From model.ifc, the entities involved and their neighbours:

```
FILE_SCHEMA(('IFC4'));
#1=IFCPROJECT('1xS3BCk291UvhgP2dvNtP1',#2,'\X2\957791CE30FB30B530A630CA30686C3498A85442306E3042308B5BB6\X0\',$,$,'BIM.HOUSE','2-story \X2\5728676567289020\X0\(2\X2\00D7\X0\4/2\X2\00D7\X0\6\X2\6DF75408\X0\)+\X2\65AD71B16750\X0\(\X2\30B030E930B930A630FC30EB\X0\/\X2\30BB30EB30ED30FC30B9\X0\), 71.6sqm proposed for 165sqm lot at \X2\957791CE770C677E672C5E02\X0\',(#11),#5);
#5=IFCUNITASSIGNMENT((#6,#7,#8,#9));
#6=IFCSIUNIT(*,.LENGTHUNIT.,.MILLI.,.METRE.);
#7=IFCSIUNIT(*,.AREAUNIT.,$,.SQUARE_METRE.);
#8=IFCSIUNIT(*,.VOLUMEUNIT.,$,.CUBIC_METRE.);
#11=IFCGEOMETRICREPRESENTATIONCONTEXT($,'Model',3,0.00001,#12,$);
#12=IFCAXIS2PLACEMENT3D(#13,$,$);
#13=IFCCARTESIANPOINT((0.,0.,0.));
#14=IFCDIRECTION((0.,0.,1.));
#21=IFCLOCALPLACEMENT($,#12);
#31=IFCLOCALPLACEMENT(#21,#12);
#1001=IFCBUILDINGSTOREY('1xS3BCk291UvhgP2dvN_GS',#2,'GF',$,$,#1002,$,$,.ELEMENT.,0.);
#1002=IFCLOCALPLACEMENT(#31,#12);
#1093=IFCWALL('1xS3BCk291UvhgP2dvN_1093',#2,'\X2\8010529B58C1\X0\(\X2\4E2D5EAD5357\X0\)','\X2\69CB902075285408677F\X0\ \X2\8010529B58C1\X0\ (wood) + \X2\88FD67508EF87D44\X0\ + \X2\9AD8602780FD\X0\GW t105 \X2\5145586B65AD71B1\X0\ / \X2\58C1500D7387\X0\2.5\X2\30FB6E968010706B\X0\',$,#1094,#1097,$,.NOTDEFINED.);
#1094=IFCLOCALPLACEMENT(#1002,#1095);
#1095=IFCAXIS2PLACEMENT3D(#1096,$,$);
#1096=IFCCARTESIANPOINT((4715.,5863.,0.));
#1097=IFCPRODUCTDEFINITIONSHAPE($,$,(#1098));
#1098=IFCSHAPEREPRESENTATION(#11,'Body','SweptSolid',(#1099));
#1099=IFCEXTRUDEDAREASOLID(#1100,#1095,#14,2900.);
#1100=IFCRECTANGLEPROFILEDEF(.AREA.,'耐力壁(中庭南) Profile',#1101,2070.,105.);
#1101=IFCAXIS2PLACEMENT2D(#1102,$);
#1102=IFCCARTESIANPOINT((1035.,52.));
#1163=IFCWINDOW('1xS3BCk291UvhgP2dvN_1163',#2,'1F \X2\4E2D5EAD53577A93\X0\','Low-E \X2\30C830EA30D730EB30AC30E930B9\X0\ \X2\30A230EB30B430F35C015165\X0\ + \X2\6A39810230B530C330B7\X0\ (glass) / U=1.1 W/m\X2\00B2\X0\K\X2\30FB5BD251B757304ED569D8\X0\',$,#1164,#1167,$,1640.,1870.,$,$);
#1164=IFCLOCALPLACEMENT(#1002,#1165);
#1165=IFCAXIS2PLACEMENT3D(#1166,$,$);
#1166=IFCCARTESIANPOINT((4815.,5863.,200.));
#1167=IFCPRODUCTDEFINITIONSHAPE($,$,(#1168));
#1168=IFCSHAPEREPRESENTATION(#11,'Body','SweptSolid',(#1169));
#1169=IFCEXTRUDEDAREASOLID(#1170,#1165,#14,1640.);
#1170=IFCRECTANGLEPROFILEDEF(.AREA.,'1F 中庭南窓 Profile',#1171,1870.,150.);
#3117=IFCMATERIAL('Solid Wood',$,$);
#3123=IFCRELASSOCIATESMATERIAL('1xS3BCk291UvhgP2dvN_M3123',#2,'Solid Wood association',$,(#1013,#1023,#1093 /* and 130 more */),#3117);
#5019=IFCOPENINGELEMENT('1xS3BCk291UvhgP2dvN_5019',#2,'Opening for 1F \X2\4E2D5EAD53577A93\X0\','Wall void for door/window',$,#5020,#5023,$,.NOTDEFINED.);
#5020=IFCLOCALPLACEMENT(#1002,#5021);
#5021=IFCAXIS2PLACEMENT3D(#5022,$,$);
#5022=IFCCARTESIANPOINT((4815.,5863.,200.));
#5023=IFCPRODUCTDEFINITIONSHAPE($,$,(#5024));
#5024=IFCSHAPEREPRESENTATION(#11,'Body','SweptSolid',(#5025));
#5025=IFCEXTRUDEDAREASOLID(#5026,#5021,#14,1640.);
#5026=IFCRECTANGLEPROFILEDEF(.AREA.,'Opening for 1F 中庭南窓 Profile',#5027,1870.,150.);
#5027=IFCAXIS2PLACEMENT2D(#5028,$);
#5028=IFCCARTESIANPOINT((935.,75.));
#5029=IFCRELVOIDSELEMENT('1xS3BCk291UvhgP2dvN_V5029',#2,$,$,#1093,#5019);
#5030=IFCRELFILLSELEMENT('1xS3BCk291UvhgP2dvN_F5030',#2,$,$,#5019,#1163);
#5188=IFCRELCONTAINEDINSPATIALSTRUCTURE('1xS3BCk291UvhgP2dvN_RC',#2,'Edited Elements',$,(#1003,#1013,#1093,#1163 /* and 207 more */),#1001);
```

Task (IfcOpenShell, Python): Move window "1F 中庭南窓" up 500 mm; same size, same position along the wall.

```python
import numpy as np
import ifcopenshell
import ifcopenshell.api.geometry
import ifcopenshell.util.placement
import ifcopenshell.util.unit

model = ifcopenshell.open("model.ifc")
unit_scale = ifcopenshell.util.unit.calculate_unit_scale(model)

window = model.by_guid("1xS3BCk291UvhgP2dvN_1163")
opening = window.FillsVoids[0].RelatingOpeningElement
dz = 0.5 / unit_scale

shift = np.array([0.0, 0.0, dz])
# The window is not placed relative to its opening, so move both.
for product in (opening, window):
    matrix = ifcopenshell.util.placement.get_local_placement(product.ObjectPlacement)
    matrix[:3, 3] += shift
    ifcopenshell.api.geometry.edit_object_placement(model, product=product, matrix=matrix, is_si=False)

print(f"moved by {dz * unit_scale:+.3f} m")

model.write("model_updated.ifc")
```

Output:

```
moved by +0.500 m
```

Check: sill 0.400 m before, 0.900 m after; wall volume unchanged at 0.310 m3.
